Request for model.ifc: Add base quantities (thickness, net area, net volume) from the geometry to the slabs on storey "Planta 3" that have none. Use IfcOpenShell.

First a look at what the model holds.

```python
import ifcopenshell
import ifcopenshell.util.element
import ifcopenshell.util.unit

model = ifcopenshell.open("model.ifc")
print(model.schema)
for unit_type in ("LENGTHUNIT", "AREAUNIT", "VOLUMEUNIT"):
    print(unit_type, ifcopenshell.util.unit.calculate_unit_scale(model, unit_type))
storey = next(s for s in model.by_type("IfcBuildingStorey") if s.Name == "Planta 3")
slabs = [e for e in ifcopenshell.util.element.get_decomposition(storey) if e.is_a("IfcSlab")]
for e in sorted(slabs, key=lambda e: e.id()):
    print(e.id(), e.is_a(), e.Name, list(ifcopenshell.util.element.get_psets(e, qtos_only=True)), sep=" | ")
```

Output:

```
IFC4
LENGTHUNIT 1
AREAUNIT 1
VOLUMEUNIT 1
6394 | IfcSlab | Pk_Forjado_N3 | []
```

```python
import ifcopenshell
import ifcopenshell.api.pset
import ifcopenshell.geom
import ifcopenshell.util.element
import ifcopenshell.util.shape
import ifcopenshell.util.unit

model = ifcopenshell.open("model.ifc")
unit_scale = ifcopenshell.util.unit.calculate_unit_scale(model)
area_scale = ifcopenshell.util.unit.calculate_unit_scale(model, "AREAUNIT")
volume_scale = ifcopenshell.util.unit.calculate_unit_scale(model, "VOLUMEUNIT")
settings = ifcopenshell.geom.settings()

storey = next(s for s in model.by_type("IfcBuildingStorey") if s.Name == "Planta 3")
slabs = [e for e in ifcopenshell.util.element.get_decomposition(storey) if e.is_a("IfcSlab")]

for e in sorted(slabs, key=lambda e: e.id()):
    if ifcopenshell.util.element.get_psets(e, qtos_only=True, should_inherit=False):
        continue
    # Geometry comes back in metres, in the element's own axes.
    shape = ifcopenshell.geom.create_shape(settings, e)
    values = {
        "Width": ifcopenshell.util.shape.get_z(shape.geometry) / unit_scale,
        "NetArea": ifcopenshell.util.shape.get_footprint_area(shape.geometry) / area_scale,
        "NetVolume": ifcopenshell.util.shape.get_volume(shape.geometry) / volume_scale,
    }
    qto = ifcopenshell.api.pset.add_qto(model, product=e, name="Qto_SlabBaseQuantities")
    ifcopenshell.api.pset.edit_qto(model, qto=qto, properties=values)
    print(e.id(), {k: round(v, 3) for k, v in values.items()})

model.write("model_v2.ifc")
```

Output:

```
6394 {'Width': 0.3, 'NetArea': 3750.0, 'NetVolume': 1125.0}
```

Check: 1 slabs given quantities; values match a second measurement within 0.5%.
